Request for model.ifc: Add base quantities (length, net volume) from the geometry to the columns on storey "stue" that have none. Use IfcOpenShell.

First a look at what the model holds.

```python
import ifcopenshell
import ifcopenshell.util.element
import ifcopenshell.util.unit

model = ifcopenshell.open("model.ifc")
print(model.schema)
for unit_type in ("LENGTHUNIT", "AREAUNIT", "VOLUMEUNIT"):
    print(unit_type, ifcopenshell.util.unit.calculate_unit_scale(model, unit_type))
storey = next(s for s in model.by_type("IfcBuildingStorey") if s.Name == "stue")
columns = [e for e in ifcopenshell.util.element.get_decomposition(storey) if e.is_a("IfcColumn")]
for e in sorted(columns, key=lambda e: e.id()):
    print(e.id(), e.is_a(), e.Name, list(ifcopenshell.util.element.get_psets(e, qtos_only=True)), sep=" | ")
```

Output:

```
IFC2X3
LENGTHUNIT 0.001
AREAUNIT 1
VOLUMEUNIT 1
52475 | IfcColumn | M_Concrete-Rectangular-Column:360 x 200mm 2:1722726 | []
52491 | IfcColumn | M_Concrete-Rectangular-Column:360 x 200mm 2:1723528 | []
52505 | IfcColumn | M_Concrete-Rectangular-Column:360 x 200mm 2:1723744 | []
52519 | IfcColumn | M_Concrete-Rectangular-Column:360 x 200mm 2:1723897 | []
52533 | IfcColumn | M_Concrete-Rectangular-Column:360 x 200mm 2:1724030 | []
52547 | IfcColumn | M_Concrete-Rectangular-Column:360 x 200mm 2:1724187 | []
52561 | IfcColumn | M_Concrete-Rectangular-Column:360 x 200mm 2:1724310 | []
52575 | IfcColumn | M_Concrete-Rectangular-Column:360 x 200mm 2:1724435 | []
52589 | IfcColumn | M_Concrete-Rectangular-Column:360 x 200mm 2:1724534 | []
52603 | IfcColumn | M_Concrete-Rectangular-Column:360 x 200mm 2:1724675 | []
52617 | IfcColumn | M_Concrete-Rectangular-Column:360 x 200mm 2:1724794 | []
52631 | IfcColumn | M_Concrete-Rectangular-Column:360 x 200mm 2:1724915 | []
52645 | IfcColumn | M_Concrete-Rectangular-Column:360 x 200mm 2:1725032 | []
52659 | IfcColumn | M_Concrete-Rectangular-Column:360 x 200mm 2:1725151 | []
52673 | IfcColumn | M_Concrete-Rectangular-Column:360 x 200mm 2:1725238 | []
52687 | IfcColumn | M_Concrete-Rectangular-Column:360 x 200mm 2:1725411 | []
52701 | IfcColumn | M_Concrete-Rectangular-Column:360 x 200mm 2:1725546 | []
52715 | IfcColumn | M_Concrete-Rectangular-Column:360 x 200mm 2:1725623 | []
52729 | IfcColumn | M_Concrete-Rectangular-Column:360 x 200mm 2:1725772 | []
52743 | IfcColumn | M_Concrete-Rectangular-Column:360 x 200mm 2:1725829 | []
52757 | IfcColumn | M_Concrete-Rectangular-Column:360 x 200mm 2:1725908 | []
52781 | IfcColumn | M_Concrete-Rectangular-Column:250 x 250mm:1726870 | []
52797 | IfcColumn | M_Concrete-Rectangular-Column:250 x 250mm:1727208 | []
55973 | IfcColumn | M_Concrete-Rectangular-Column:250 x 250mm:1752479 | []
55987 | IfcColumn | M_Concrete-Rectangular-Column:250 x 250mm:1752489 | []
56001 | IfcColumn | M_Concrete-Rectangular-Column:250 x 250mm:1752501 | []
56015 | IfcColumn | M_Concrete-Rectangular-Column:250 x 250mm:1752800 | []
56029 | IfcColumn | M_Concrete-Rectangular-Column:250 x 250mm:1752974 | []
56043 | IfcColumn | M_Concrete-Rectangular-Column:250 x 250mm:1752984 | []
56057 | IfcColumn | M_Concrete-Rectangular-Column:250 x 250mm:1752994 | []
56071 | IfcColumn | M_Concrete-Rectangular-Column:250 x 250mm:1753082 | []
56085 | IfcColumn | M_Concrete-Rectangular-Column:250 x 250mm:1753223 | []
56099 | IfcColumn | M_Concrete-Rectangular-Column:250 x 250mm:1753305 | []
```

```python
import ifcopenshell
import ifcopenshell.api.pset
import ifcopenshell.geom
import ifcopenshell.util.element
import ifcopenshell.util.shape
import ifcopenshell.util.unit

model = ifcopenshell.open("model.ifc")
unit_scale = ifcopenshell.util.unit.calculate_unit_scale(model)
volume_scale = ifcopenshell.util.unit.calculate_unit_scale(model, "VOLUMEUNIT")
settings = ifcopenshell.geom.settings()

storey = next(s for s in model.by_type("IfcBuildingStorey") if s.Name == "stue")
columns = [e for e in ifcopenshell.util.element.get_decomposition(storey) if e.is_a("IfcColumn")]

for e in sorted(columns, key=lambda e: e.id()):
    if ifcopenshell.util.element.get_psets(e, qtos_only=True, should_inherit=False):
        continue
    # Geometry comes back in metres, in the element's own axes.
    shape = ifcopenshell.geom.create_shape(settings, e)
    values = {
        "Length": ifcopenshell.util.shape.get_z(shape.geometry) / unit_scale,
        "NetVolume": ifcopenshell.util.shape.get_volume(shape.geometry) / volume_scale,
    }
    qto = ifcopenshell.api.pset.add_qto(model, product=e, name="BaseQuantities")
    ifcopenshell.api.pset.edit_qto(model, qto=qto, properties=values)
    print(e.id(), {k: round(v, 3) for k, v in values.items()})

model.write("model_rev.ifc")
```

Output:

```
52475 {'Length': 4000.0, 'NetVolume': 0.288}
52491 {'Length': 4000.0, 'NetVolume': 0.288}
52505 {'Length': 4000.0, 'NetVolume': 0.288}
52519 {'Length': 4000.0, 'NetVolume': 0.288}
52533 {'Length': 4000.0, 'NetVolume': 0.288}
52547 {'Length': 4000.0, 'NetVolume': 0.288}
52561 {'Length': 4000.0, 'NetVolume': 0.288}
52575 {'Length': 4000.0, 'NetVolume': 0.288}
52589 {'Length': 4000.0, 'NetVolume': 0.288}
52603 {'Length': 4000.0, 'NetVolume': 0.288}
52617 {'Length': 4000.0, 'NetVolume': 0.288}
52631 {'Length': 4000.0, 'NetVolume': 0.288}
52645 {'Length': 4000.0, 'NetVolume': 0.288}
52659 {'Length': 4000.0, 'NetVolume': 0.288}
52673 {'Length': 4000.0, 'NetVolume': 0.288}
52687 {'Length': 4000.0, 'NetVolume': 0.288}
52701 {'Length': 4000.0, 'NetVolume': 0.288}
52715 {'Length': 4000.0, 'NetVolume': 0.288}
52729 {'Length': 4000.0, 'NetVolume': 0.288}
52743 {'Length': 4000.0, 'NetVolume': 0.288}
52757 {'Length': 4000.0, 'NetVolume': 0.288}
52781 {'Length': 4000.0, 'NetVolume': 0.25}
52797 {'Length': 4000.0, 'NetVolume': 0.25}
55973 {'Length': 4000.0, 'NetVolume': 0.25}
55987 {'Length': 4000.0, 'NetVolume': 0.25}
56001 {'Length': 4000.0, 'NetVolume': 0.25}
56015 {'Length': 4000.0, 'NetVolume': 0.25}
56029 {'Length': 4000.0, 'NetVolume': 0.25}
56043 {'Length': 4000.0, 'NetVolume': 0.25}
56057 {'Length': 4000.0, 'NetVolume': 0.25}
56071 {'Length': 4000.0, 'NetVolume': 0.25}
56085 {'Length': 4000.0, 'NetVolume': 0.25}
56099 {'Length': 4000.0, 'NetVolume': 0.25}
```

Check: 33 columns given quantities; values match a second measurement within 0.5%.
